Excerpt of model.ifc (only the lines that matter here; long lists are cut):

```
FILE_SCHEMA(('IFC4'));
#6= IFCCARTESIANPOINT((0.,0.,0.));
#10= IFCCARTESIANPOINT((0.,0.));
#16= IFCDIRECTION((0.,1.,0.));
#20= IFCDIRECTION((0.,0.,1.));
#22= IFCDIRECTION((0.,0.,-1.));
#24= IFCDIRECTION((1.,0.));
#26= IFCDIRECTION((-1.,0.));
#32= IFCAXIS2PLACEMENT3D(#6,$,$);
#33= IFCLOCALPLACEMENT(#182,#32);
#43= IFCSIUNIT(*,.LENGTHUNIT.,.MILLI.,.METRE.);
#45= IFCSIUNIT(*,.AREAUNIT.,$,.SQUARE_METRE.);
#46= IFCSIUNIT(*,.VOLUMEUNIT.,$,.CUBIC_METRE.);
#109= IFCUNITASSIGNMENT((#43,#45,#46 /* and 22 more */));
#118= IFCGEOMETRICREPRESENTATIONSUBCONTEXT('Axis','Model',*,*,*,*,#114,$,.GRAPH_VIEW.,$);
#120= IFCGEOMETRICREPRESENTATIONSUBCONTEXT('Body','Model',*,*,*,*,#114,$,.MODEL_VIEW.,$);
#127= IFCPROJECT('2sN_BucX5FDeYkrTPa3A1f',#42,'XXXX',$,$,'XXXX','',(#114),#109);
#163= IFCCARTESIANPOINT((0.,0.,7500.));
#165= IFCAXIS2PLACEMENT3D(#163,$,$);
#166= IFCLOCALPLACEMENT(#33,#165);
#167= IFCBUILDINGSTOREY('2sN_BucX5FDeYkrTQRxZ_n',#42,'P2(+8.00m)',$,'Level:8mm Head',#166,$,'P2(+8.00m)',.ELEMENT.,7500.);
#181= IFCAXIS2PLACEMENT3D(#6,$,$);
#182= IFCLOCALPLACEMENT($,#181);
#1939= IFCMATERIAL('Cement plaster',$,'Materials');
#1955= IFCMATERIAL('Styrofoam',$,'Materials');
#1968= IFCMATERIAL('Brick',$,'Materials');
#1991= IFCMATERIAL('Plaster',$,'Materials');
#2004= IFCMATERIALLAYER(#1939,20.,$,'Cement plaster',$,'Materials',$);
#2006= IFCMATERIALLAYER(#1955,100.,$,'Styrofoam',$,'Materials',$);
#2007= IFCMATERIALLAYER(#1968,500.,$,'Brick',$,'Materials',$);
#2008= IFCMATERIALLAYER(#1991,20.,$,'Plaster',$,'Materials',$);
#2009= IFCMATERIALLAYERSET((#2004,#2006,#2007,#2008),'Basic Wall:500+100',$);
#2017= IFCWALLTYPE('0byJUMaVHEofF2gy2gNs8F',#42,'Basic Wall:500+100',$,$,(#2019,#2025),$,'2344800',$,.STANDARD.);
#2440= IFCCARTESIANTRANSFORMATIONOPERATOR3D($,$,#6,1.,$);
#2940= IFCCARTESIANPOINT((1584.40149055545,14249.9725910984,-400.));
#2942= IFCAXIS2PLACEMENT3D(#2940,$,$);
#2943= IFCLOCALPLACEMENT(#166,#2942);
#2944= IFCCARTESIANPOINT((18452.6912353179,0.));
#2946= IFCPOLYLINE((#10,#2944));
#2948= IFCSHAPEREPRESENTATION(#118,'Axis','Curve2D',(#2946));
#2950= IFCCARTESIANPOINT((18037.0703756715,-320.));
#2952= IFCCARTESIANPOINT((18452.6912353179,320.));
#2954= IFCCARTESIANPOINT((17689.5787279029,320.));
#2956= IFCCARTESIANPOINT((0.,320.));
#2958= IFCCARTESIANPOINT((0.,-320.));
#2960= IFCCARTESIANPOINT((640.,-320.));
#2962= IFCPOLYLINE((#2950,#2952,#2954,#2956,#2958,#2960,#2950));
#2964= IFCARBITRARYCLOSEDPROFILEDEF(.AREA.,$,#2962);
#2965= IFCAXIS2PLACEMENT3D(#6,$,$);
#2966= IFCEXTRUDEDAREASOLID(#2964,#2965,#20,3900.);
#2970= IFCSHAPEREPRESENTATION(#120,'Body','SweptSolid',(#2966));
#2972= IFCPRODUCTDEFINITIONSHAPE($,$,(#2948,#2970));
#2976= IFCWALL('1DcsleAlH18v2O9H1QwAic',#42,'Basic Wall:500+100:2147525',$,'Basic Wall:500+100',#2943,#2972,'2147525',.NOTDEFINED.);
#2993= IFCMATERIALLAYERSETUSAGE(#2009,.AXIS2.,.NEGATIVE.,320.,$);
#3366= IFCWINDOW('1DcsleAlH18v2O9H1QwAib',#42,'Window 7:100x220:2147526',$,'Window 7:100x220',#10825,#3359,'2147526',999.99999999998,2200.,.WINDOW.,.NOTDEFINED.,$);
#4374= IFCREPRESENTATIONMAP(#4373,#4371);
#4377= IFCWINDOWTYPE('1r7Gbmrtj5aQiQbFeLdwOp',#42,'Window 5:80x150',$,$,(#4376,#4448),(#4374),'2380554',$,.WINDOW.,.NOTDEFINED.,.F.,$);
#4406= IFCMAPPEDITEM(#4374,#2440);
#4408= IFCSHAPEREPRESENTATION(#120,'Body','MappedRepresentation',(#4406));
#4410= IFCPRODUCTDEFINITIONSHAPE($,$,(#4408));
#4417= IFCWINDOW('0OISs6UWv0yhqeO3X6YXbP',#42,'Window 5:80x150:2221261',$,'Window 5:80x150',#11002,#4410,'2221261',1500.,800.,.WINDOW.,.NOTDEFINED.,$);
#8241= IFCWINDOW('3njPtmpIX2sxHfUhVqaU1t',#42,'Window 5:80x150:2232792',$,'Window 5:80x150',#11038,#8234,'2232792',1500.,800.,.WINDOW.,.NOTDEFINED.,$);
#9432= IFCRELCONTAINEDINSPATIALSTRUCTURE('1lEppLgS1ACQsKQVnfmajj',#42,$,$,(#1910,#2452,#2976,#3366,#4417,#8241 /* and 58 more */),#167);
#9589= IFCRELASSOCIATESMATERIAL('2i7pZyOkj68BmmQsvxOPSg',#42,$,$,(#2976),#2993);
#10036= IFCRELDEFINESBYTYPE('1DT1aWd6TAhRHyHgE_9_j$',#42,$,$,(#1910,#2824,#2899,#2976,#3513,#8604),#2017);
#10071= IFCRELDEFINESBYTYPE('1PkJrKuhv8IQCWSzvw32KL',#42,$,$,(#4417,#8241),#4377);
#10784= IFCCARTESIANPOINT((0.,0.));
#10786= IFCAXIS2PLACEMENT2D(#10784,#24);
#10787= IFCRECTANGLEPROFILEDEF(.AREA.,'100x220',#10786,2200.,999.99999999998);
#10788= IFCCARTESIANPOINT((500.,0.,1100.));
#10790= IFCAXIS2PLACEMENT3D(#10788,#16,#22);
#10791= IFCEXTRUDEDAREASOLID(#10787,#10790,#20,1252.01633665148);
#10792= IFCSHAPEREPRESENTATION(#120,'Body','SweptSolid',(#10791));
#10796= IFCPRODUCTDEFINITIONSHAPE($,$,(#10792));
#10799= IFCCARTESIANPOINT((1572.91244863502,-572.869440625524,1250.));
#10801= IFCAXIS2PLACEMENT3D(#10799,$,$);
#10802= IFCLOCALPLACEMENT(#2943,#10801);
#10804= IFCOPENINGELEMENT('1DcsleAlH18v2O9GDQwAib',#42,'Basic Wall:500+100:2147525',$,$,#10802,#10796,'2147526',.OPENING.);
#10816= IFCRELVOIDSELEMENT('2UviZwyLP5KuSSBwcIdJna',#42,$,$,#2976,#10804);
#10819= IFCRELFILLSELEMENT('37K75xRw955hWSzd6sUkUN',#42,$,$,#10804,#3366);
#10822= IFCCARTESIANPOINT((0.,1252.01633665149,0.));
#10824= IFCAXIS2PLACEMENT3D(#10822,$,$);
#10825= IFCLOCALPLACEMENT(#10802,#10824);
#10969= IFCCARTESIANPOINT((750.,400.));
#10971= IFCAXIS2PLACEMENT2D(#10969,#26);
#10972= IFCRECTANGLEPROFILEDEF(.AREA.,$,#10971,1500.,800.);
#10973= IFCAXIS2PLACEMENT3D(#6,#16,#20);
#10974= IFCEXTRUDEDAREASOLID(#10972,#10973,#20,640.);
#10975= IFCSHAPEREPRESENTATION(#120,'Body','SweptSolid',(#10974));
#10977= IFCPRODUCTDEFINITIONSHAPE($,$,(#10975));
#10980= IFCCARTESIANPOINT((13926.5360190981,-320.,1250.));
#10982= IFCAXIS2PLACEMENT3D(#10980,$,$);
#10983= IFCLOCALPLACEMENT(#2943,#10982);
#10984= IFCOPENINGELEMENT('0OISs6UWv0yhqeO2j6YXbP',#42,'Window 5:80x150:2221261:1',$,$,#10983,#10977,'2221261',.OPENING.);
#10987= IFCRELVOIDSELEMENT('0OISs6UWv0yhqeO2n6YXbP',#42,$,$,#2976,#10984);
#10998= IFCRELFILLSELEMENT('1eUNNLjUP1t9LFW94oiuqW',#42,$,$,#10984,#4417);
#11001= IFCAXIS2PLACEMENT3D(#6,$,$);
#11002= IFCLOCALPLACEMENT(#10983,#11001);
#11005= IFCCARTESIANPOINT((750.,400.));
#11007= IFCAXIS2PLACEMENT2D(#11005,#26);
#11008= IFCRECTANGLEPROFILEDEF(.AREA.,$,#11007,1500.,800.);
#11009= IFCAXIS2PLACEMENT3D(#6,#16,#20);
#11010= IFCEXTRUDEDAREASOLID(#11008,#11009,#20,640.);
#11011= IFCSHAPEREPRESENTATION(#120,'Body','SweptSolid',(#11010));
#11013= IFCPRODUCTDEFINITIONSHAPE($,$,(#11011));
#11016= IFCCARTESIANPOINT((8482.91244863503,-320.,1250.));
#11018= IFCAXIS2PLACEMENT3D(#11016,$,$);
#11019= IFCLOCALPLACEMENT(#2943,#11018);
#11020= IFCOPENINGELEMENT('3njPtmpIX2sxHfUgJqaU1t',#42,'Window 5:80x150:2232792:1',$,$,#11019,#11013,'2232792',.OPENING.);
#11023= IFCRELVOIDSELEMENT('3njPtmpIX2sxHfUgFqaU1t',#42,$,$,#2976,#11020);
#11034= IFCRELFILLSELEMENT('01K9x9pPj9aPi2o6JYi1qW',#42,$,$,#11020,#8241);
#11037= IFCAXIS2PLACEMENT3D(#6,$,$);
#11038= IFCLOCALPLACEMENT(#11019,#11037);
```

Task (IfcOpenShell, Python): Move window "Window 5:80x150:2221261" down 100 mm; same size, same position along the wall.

```python
import numpy as np
import ifcopenshell
import ifcopenshell.api.geometry
import ifcopenshell.util.placement
import ifcopenshell.util.unit

model = ifcopenshell.open("model.ifc")
unit_scale = ifcopenshell.util.unit.calculate_unit_scale(model)

window = model.by_id(4417)
opening = window.FillsVoids[0].RelatingOpeningElement
dz = -100.0

shift = np.array([0.0, 0.0, dz])
# The window is placed relative to its opening, so it follows when the opening moves.
matrix = ifcopenshell.util.placement.get_local_placement(opening.ObjectPlacement)
matrix[:3, 3] += shift
ifcopenshell.api.geometry.edit_object_placement(
    model, product=opening, matrix=matrix, is_si=False, should_transform_children=True
)

print(f"moved by {dz * unit_scale:+.3f} m")

model.write("model_v2.ifc")
```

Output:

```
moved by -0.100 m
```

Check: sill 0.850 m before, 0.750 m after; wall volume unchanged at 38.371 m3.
